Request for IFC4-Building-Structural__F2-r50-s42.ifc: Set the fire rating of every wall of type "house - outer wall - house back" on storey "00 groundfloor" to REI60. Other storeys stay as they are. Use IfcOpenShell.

First a look at what the model holds.

```python
import ifcopenshell
import ifcopenshell.util.element

model = ifcopenshell.open("IFC4-Building-Structural__F2-r50-s42.ifc")
print(model.schema)
storey = next(s for s in model.by_type("IfcBuildingStorey") if s.Name == "00 groundfloor")
walls = [e for e in ifcopenshell.util.element.get_decomposition(storey) if e.is_a("IfcWall")]
seen = {}
for e in walls:
    element_type = ifcopenshell.util.element.get_type(e)
    key = (element_type.Name if element_type != e and element_type else None, ifcopenshell.util.element.get_pset(e, "Pset_WallCommon", "FireRating"))
    seen[key] = seen.get(key, 0) + 1
for (name, value), count in sorted(seen.items(), key=str):
    print(count, "x", name, "|", value)
```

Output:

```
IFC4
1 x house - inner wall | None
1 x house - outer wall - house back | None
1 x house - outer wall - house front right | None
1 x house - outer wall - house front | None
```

```python
import ifcopenshell
import ifcopenshell.api.pset
import ifcopenshell.util.element

model = ifcopenshell.open("IFC4-Building-Structural__F2-r50-s42.ifc")

storey = next(s for s in model.by_type("IfcBuildingStorey") if s.Name == "00 groundfloor")
walls = [e for e in ifcopenshell.util.element.get_decomposition(storey) if e.is_a("IfcWall")]

count = 0
for e in walls:
    element_type = ifcopenshell.util.element.get_type(e)
    if element_type in (None, e) or element_type.Name != "house - outer wall - house back":
        continue
    # add_pset returns the element's existing set when there is one.
    pset = ifcopenshell.api.pset.add_pset(model, product=e, name="Pset_WallCommon")
    ifcopenshell.api.pset.edit_pset(model, pset=pset, properties={"FireRating": "REI60"})
    count += 1

print(count, "walls updated")

model.write("IFC4-Building-Structural__F2-r50-s42_updated.ifc")
```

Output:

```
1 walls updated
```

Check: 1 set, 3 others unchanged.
